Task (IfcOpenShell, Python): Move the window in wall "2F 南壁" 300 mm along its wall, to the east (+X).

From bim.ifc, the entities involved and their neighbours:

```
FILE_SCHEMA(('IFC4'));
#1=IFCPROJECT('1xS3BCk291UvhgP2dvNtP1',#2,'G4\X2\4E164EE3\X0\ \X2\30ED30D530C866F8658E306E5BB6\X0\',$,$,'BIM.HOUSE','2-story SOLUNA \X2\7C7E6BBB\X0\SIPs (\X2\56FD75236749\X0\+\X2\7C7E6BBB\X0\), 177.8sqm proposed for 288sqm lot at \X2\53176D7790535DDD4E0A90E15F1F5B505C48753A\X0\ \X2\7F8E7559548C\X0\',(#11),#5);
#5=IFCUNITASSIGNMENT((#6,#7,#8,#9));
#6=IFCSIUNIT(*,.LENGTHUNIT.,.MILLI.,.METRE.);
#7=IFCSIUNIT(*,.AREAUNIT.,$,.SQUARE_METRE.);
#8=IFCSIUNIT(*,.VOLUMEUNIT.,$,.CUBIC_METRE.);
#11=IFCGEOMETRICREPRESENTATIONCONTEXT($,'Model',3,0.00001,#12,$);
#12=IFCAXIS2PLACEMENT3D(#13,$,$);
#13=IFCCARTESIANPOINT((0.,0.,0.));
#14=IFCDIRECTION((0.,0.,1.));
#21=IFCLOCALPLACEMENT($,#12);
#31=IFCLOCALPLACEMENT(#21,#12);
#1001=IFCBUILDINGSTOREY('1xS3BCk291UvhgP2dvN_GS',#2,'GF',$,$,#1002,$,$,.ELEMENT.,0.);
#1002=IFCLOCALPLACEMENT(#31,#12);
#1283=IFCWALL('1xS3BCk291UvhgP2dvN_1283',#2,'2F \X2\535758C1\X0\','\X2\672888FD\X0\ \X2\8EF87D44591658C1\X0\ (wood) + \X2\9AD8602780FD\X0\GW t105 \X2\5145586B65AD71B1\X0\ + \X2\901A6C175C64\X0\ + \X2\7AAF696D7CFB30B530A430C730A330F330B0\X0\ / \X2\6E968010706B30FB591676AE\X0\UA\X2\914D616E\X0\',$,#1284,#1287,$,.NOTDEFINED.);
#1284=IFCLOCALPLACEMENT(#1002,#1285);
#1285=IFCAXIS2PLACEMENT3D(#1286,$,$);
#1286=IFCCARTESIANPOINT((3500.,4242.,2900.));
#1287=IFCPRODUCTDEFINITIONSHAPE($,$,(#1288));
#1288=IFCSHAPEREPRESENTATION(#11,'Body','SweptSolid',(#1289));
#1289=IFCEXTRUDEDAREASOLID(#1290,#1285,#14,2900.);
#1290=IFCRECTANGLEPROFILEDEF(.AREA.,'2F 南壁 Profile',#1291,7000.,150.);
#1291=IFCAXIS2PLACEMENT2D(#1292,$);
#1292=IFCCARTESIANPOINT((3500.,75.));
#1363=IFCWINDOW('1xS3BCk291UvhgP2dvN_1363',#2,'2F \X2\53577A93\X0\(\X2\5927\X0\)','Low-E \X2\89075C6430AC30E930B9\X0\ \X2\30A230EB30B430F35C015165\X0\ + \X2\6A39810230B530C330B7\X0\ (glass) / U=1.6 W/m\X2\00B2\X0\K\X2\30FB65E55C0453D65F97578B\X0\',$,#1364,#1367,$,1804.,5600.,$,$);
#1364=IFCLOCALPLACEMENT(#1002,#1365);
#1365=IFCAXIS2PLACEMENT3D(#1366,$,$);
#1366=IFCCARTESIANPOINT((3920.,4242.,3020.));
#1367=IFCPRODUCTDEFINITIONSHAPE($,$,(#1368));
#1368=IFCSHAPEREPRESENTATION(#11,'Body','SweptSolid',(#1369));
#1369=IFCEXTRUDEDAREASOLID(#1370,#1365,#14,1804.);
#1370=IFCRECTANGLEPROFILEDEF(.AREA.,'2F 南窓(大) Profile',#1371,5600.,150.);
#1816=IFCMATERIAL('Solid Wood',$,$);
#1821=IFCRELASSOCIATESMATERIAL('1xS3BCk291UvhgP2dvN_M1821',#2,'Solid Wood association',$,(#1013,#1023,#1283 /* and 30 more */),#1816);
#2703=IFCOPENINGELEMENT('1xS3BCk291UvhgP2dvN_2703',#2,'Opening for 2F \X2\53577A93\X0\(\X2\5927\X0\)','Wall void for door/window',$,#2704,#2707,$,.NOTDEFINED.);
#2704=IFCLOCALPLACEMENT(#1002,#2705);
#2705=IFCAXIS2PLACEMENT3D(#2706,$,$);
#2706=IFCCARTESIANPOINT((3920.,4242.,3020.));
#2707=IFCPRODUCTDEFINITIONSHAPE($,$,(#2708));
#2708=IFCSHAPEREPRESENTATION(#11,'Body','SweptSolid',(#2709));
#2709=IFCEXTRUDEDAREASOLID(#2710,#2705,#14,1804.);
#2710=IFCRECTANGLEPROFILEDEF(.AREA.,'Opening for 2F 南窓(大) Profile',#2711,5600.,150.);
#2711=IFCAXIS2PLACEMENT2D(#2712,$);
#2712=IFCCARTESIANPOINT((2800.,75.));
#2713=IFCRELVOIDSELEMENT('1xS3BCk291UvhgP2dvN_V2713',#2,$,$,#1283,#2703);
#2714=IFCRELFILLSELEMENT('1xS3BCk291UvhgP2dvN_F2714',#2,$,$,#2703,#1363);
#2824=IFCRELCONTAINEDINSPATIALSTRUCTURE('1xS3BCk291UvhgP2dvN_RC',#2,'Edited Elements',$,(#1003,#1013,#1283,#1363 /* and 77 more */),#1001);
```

```python
import ifcopenshell
import ifcopenshell.api.geometry
import ifcopenshell.util.placement
import ifcopenshell.util.unit

model = ifcopenshell.open("bim.ifc")
unit_scale = ifcopenshell.util.unit.calculate_unit_scale(model)

window = model.by_guid("1xS3BCk291UvhgP2dvN_1363")
opening = window.FillsVoids[0].RelatingOpeningElement
wall = opening.VoidsElements[0].RelatingBuildingElement

wall_matrix = ifcopenshell.util.placement.get_local_placement(wall.ObjectPlacement)
shift = wall_matrix[:3, 0] * 0.3 / unit_scale
before = ifcopenshell.util.placement.get_local_placement(window.ObjectPlacement)[:3, 3].copy()

# The window is not placed relative to its opening, so move both.
for product in (opening, window):
    matrix = ifcopenshell.util.placement.get_local_placement(product.ObjectPlacement)
    matrix[:3, 3] += shift
    ifcopenshell.api.geometry.edit_object_placement(model, product=product, matrix=matrix, is_si=False)

after = ifcopenshell.util.placement.get_local_placement(window.ObjectPlacement)[:3, 3]
print("window moved by", (after - before).round(3) + 0.0)

model.write("bim_rev.ifc")
```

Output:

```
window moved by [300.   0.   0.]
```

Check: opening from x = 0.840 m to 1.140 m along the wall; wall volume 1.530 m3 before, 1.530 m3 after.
